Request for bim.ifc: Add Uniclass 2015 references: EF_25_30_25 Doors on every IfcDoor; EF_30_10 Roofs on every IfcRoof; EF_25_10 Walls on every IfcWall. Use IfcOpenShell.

First a look at what the model holds.

```python
import ifcopenshell

model = ifcopenshell.open("bim.ifc")
print(model.schema)
print("classifications:", [c.Name for c in model.by_type("IfcClassification")])
for ifc_class in ("IfcDoor", "IfcRoof", "IfcStair", "IfcWall", "IfcWindow"):
    print(ifc_class, len(model.by_type(ifc_class)))
```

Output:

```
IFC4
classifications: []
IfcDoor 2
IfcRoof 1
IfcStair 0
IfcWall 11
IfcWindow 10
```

```python
import ifcopenshell
import ifcopenshell.api.classification

model = ifcopenshell.open("bim.ifc")

system = ifcopenshell.api.classification.add_classification(model, classification="Uniclass 2015")

codes = {
    "IfcDoor": ("EF_25_30_25", "Doors"),
    "IfcRoof": ("EF_30_10", "Roofs"),
    "IfcWall": ("EF_25_10", "Walls"),
}
for ifc_class, (code, name) in codes.items():
    products = model.by_type(ifc_class)
    ifcopenshell.api.classification.add_reference(
        model, products=products, classification=system, identification=code, name=name
    )
    print(code, len(products))

model.write("bim_rev.ifc")
```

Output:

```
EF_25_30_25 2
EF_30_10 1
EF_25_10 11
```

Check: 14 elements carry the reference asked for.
